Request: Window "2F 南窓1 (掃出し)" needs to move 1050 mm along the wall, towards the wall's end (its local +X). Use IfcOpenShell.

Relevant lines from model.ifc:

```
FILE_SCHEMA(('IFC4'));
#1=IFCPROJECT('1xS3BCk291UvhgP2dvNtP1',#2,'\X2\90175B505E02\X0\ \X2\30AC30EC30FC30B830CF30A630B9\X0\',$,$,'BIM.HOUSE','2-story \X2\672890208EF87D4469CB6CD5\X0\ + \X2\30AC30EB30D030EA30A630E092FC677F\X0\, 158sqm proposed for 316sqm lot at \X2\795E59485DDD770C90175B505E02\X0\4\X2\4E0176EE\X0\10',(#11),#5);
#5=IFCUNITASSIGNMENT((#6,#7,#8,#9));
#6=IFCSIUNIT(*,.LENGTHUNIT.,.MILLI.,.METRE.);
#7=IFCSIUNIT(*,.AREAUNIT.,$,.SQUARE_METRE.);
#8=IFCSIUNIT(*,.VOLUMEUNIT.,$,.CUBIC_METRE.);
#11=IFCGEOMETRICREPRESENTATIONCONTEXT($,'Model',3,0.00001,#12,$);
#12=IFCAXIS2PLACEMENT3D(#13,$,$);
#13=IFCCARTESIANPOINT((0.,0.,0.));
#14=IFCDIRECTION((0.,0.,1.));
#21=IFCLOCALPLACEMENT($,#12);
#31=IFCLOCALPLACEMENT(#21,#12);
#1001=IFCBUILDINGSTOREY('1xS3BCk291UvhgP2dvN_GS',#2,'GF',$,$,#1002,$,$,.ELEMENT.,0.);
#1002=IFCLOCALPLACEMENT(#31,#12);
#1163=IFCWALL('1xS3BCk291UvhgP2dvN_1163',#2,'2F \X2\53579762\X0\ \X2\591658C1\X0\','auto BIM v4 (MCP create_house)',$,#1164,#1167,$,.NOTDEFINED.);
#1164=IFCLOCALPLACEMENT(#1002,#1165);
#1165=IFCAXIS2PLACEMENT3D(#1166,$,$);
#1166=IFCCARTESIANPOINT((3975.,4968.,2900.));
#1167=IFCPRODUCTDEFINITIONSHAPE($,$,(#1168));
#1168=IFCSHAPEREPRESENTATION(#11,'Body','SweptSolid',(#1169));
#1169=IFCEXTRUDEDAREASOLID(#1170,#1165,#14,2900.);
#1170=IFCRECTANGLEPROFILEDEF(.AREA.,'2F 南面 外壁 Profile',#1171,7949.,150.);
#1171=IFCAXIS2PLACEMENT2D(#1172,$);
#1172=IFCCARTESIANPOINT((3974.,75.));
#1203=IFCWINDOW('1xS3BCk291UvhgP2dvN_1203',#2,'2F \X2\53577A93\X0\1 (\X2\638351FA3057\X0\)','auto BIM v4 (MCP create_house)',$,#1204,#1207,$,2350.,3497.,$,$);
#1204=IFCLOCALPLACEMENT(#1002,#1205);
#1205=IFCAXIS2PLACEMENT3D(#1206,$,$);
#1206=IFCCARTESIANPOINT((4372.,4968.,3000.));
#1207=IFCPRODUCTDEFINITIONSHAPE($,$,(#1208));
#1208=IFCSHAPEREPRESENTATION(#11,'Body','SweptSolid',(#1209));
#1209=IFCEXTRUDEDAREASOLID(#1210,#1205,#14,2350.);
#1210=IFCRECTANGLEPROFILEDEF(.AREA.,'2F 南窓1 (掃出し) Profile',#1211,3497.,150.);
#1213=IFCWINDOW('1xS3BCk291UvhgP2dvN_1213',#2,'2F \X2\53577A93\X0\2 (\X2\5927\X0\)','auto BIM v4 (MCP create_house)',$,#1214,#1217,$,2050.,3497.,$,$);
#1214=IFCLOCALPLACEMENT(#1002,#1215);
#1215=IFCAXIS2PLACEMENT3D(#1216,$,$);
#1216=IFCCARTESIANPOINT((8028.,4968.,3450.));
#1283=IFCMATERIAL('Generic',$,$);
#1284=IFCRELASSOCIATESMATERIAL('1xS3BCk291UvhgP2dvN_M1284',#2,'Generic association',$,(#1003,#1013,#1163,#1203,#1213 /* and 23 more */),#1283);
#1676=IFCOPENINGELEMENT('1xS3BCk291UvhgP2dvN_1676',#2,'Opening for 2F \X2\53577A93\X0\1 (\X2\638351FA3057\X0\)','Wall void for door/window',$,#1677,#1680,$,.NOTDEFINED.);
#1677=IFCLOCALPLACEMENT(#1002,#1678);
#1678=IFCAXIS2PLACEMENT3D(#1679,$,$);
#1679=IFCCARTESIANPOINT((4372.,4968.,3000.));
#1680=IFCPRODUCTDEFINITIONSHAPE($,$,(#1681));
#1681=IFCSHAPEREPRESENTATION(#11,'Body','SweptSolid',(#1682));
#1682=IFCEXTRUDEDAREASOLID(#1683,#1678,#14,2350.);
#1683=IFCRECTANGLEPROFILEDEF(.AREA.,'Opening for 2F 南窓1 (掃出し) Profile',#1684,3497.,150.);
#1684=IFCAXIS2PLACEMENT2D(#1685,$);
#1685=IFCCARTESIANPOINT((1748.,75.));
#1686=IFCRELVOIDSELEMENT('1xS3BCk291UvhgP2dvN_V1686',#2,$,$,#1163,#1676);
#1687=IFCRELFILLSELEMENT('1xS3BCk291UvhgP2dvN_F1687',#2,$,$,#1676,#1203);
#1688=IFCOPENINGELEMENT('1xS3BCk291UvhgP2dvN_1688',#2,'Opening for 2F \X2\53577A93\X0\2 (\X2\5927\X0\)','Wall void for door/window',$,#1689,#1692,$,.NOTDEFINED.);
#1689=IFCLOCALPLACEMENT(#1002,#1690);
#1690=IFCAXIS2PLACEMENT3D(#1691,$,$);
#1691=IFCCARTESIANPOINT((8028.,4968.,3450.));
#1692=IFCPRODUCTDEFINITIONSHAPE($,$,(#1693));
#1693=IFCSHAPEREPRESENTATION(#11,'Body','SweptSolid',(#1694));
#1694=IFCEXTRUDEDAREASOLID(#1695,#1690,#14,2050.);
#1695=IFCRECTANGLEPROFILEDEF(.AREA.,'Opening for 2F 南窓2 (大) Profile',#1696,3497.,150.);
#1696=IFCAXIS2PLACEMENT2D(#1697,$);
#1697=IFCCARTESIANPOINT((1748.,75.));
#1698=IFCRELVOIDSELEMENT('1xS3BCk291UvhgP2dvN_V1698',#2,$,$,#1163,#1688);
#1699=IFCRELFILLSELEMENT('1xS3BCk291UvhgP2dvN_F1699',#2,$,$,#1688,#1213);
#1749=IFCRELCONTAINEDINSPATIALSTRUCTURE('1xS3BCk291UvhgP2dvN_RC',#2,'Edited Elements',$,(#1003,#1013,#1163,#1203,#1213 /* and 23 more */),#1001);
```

```python
import ifcopenshell
import ifcopenshell.api.geometry
import ifcopenshell.util.placement
import ifcopenshell.util.unit

model = ifcopenshell.open("model.ifc")
unit_scale = ifcopenshell.util.unit.calculate_unit_scale(model)

window = model.by_guid("1xS3BCk291UvhgP2dvN_1203")
opening = window.FillsVoids[0].RelatingOpeningElement
wall = opening.VoidsElements[0].RelatingBuildingElement

wall_matrix = ifcopenshell.util.placement.get_local_placement(wall.ObjectPlacement)
shift = wall_matrix[:3, 0] * 1.05 / unit_scale
before = ifcopenshell.util.placement.get_local_placement(window.ObjectPlacement)[:3, 3].copy()

# The window is not placed relative to its opening, so move both.
for product in (opening, window):
    matrix = ifcopenshell.util.placement.get_local_placement(product.ObjectPlacement)
    matrix[:3, 3] += shift
    ifcopenshell.api.geometry.edit_object_placement(model, product=product, matrix=matrix, is_si=False)

after = ifcopenshell.util.placement.get_local_placement(window.ObjectPlacement)[:3, 3]
print("window moved by", (after - before).round(3) + 0.0)

model.write("model_edited.ifc")
```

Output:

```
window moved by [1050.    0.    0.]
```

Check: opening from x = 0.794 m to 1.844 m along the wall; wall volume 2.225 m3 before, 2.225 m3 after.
